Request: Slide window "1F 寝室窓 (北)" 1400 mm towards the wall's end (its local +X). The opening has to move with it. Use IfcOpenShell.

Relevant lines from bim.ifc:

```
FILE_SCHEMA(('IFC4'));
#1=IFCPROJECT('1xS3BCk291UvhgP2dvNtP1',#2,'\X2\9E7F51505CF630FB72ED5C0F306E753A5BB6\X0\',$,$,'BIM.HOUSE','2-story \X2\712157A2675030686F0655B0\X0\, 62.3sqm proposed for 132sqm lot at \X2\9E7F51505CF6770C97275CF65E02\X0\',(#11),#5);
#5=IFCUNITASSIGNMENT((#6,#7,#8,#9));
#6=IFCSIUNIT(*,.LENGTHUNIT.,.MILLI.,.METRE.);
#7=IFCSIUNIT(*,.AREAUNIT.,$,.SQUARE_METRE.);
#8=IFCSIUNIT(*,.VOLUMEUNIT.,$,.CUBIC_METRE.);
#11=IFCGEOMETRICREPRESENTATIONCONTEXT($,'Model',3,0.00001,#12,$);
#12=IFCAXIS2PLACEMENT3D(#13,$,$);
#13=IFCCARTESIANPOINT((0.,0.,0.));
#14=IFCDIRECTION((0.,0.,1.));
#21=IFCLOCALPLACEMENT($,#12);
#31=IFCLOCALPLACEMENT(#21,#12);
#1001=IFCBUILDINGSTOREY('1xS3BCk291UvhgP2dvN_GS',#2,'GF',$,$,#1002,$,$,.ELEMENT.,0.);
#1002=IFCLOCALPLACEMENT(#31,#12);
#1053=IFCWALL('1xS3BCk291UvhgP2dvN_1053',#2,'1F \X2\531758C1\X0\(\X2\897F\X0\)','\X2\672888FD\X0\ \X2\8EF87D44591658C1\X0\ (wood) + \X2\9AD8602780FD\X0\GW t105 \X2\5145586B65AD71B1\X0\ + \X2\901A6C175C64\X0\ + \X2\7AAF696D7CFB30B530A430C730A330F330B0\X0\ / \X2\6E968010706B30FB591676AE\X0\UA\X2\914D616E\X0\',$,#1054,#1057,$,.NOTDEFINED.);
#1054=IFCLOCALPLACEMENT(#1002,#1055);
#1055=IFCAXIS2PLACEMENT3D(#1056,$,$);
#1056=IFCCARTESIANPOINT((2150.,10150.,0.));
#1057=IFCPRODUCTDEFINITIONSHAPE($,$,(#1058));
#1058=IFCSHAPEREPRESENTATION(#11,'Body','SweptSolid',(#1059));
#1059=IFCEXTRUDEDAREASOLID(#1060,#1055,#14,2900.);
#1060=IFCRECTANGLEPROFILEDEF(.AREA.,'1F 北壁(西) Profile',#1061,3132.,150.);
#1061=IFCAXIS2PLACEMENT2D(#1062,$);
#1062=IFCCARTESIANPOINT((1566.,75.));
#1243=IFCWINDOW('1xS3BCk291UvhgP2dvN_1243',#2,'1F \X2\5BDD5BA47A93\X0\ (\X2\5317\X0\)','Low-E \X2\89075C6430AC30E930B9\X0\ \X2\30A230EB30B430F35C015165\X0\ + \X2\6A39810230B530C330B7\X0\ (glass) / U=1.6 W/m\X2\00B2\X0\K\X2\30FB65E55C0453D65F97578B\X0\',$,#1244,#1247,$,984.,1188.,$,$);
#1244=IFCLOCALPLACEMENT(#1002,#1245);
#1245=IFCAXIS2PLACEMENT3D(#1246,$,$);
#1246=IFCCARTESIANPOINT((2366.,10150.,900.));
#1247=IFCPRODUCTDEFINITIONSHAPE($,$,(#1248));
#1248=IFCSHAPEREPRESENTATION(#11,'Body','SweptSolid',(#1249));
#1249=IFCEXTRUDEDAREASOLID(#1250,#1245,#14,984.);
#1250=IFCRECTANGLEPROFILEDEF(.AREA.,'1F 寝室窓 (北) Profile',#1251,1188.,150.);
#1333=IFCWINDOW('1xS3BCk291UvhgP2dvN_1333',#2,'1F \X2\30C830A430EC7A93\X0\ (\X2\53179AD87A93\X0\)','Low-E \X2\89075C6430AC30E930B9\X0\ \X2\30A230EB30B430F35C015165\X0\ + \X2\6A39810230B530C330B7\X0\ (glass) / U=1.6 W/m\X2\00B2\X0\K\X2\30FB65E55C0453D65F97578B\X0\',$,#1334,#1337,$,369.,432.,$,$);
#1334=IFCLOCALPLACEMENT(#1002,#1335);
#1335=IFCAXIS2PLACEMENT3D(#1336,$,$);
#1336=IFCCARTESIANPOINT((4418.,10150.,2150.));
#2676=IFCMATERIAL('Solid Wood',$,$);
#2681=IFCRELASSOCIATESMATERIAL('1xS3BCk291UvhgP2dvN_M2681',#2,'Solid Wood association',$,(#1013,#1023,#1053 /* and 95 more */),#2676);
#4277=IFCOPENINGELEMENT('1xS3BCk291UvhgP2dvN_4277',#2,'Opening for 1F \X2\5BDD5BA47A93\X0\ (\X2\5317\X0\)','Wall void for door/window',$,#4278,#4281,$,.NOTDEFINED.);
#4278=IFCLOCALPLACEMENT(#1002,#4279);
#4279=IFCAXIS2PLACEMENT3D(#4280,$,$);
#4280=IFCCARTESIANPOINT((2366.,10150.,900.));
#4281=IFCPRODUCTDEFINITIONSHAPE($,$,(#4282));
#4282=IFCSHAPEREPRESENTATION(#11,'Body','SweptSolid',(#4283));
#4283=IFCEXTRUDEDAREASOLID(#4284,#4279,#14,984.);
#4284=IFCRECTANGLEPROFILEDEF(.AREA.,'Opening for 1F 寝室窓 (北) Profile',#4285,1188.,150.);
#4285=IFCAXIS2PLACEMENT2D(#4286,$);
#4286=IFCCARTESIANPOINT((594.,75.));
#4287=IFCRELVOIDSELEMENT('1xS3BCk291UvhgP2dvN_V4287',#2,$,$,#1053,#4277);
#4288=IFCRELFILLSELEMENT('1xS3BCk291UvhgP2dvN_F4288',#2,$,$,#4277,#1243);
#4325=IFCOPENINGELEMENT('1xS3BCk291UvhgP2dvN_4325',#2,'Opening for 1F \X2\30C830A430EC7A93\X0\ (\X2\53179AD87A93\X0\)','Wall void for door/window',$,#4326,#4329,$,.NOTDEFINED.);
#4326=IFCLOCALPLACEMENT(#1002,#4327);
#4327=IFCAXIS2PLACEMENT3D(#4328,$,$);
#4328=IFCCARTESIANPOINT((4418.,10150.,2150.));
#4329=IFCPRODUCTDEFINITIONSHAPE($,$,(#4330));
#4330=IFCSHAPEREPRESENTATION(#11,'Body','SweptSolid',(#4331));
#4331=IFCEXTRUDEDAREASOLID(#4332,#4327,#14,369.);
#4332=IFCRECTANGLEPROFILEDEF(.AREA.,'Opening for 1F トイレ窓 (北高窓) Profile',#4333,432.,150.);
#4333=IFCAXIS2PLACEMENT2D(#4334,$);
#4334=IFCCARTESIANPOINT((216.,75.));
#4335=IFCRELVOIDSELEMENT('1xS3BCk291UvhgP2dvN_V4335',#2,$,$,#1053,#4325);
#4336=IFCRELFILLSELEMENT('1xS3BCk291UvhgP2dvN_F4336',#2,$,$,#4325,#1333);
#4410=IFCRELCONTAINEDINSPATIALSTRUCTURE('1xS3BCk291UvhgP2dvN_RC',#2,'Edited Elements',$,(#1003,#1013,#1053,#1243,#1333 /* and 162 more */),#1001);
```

```python
import ifcopenshell
import ifcopenshell.api.geometry
import ifcopenshell.util.placement

model = ifcopenshell.open("bim.ifc")

window = model.by_guid("1xS3BCk291UvhgP2dvN_1243")
opening = window.FillsVoids[0].RelatingOpeningElement
wall = opening.VoidsElements[0].RelatingBuildingElement

wall_matrix = ifcopenshell.util.placement.get_local_placement(wall.ObjectPlacement)
shift = wall_matrix[:3, 0] * 1400.0
before = ifcopenshell.util.placement.get_local_placement(window.ObjectPlacement)[:3, 3].copy()

# The window is not placed relative to its opening, so move both.
for product in (opening, window):
    matrix = ifcopenshell.util.placement.get_local_placement(product.ObjectPlacement)
    matrix[:3, 3] += shift
    ifcopenshell.api.geometry.edit_object_placement(model, product=product, matrix=matrix, is_si=False)

after = ifcopenshell.util.placement.get_local_placement(window.ObjectPlacement)[:3, 3]
print("window moved by", (after - before).round(3) + 0.0)

model.write("bim_updated.ifc")
```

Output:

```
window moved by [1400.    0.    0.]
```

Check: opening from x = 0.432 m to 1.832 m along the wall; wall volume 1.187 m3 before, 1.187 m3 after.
